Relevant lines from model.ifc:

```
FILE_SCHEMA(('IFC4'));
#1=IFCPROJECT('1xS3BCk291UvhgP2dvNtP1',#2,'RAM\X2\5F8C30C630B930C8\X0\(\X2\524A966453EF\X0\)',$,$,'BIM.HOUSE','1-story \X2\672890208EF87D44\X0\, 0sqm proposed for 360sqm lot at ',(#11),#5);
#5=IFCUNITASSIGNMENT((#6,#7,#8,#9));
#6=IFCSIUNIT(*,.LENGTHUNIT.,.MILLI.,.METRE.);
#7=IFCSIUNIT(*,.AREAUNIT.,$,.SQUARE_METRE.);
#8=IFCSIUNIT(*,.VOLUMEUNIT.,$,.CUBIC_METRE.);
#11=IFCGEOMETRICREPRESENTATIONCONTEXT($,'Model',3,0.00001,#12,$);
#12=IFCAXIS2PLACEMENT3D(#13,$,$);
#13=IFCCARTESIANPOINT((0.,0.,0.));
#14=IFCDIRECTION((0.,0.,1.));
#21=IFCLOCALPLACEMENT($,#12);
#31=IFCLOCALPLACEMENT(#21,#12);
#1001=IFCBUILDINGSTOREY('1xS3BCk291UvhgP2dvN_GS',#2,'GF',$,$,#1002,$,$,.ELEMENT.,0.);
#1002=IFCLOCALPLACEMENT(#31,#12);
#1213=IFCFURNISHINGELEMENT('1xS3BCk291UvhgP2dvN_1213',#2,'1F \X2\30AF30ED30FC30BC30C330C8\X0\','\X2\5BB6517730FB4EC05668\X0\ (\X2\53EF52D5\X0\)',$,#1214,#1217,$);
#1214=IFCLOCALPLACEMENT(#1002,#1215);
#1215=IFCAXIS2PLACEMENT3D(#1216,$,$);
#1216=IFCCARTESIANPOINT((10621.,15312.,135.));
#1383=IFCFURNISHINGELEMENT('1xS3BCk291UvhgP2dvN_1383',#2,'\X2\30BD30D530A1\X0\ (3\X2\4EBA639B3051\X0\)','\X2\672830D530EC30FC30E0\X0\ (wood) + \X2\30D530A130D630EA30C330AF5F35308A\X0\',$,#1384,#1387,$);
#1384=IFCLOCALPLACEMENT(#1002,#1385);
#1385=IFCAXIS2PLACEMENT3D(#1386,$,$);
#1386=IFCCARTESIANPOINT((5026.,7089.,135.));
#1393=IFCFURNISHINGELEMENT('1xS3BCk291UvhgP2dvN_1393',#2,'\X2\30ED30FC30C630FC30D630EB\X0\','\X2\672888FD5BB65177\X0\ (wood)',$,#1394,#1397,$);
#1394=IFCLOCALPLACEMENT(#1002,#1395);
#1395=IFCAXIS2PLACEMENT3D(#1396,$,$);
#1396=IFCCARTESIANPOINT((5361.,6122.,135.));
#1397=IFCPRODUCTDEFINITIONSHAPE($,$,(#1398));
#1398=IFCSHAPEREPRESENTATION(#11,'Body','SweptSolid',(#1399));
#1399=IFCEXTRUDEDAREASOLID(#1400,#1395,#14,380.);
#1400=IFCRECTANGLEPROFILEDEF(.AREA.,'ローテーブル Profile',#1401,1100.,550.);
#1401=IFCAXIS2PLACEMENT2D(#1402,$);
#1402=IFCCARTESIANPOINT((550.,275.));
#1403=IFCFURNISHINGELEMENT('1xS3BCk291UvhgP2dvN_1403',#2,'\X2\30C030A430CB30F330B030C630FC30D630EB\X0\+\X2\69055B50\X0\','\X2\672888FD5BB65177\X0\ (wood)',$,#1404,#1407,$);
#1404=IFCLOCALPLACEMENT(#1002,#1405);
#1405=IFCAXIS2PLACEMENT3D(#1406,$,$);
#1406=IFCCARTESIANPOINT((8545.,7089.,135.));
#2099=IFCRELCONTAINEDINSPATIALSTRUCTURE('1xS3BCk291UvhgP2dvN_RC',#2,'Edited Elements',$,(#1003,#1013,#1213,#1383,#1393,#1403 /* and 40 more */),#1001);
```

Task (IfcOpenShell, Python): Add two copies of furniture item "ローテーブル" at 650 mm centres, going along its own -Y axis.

```python
import ifcopenshell
import ifcopenshell.api.geometry
import ifcopenshell.api.root
import ifcopenshell.util.element
import ifcopenshell.util.placement
import ifcopenshell.util.unit

model = ifcopenshell.open("model.ifc")
unit_scale = ifcopenshell.util.unit.calculate_unit_scale(model)


def reuse_history(source, copy):
    """copy_class also copies each property set's owner history, people and application; keep the originals."""
    for rel in copy.IsDefinedBy:
        if rel.is_a("IfcRelDefinesByProperties") and (history := rel.RelatingPropertyDefinition.OwnerHistory):
            rel.RelatingPropertyDefinition.OwnerHistory = source.OwnerHistory
            ifcopenshell.util.element.remove_deep2(model, history)


source = model.by_guid("1xS3BCk291UvhgP2dvN_1393")
base = ifcopenshell.util.placement.get_local_placement(source.ObjectPlacement)
step = -base[:3, 1] * 0.65 / unit_scale

for i in range(1, 3):
    copy = ifcopenshell.api.root.copy_class(model, product=source)
    copy.Representation = ifcopenshell.util.element.copy_deep(
        model, source.Representation, exclude=["IfcGeometricRepresentationContext", "IfcRepresentationMap"]
    )
    reuse_history(source, copy)
    matrix = base.copy()
    matrix[:3, 3] += i * step
    print("added at", matrix[:3, 3].round(3) + 0.0)
    ifcopenshell.api.geometry.edit_object_placement(model, product=copy, matrix=matrix, is_si=False)

model.write("model_edited.ifc")
```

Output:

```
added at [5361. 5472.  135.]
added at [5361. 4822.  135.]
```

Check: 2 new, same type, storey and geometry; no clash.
